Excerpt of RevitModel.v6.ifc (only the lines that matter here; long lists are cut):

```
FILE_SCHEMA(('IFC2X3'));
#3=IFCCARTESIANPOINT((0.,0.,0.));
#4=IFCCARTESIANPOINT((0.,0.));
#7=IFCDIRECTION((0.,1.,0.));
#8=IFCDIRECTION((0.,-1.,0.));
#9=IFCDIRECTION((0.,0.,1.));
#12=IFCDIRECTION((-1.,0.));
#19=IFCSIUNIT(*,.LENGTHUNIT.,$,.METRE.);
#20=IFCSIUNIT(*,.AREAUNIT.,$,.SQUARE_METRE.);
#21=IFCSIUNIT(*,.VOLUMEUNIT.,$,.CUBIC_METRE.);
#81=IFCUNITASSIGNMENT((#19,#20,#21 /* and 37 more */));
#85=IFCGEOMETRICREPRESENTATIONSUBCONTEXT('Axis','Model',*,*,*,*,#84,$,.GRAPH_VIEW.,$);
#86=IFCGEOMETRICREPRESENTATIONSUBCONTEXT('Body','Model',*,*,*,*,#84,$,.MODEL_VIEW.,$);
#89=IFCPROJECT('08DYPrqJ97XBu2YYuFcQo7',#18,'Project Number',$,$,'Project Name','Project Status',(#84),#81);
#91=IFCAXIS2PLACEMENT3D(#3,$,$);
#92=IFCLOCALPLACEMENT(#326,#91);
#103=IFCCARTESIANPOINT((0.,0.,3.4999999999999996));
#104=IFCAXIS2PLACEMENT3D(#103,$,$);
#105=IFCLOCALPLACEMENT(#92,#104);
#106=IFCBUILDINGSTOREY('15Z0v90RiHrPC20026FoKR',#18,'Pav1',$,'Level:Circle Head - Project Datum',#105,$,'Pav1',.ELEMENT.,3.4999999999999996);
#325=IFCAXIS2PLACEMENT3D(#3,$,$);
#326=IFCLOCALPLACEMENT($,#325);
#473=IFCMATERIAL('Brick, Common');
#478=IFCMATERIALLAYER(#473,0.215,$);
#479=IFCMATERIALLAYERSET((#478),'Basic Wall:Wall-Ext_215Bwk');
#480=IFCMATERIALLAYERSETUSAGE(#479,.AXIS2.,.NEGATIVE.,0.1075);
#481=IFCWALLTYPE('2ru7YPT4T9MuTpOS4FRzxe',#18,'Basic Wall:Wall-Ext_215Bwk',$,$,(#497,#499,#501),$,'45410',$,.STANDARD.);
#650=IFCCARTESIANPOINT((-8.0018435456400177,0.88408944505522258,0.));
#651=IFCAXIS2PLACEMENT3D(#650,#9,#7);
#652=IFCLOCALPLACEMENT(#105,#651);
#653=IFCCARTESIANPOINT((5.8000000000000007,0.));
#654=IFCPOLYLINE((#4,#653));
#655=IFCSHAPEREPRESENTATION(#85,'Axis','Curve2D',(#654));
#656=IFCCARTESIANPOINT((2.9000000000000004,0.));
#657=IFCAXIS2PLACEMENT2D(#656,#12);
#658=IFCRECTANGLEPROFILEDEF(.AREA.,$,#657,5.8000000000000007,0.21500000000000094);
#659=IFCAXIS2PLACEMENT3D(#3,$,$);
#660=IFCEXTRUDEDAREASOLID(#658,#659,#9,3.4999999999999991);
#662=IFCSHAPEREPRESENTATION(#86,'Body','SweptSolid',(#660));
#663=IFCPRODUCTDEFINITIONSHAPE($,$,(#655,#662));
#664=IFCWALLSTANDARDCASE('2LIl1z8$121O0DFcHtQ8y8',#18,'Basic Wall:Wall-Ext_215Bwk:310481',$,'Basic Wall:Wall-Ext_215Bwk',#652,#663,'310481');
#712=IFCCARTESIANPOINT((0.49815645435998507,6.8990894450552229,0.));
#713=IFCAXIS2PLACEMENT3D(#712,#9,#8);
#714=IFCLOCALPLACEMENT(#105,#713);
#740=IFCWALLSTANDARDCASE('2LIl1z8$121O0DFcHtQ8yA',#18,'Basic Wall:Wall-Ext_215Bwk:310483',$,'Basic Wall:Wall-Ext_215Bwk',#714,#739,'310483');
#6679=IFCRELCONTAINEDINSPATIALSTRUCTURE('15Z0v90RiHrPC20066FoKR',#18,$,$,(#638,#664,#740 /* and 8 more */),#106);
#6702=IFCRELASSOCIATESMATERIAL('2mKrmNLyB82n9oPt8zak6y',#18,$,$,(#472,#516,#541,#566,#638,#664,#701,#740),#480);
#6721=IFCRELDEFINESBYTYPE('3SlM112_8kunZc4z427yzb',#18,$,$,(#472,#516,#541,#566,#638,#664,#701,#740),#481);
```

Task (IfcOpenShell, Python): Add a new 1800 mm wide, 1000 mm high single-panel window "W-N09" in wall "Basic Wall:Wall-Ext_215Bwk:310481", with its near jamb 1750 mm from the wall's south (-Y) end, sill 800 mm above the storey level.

```python
import numpy as np
import ifcopenshell
import ifcopenshell.api.feature
import ifcopenshell.api.geometry
import ifcopenshell.api.root
import ifcopenshell.api.spatial
import ifcopenshell.api.type
import ifcopenshell.geom
import ifcopenshell.util.element
import ifcopenshell.util.placement
import ifcopenshell.util.representation
import ifcopenshell.util.shape
import ifcopenshell.util.unit

model = ifcopenshell.open("RevitModel.v6.ifc")
unit_scale = ifcopenshell.util.unit.calculate_unit_scale(model)
settings = ifcopenshell.geom.settings()


def volume(element):
    """Net volume in cubic metres, openings subtracted."""
    shape = ifcopenshell.geom.create_shape(settings, element)
    return ifcopenshell.util.shape.get_volume(shape.geometry)


wall = model.by_id(664)
storey = ifcopenshell.util.element.get_container(wall, ifc_class="IfcBuildingStorey")
context = ifcopenshell.util.representation.get_context(model, "Model", "Body", "MODEL_VIEW")
before = volume(wall)

width, height, from_end, sill = 1.8, 1, 1.75, 0.8  # metres

# The wall runs along its own X axis, and the end named is its -X end.
wall_shape = ifcopenshell.geom.create_shape(settings, wall)
x, y, z = ifcopenshell.util.shape.get_vertices(wall_shape.geometry).T
start = x.min() + from_end
face, thickness = float(y.min()), float(y.max() - y.min())
wall_matrix = ifcopenshell.util.placement.get_local_placement(wall.ObjectPlacement)
level = ifcopenshell.util.placement.get_local_placement(storey.ObjectPlacement)[2, 3]


def in_wall(x, y):
    """Placement at x, y metres in the wall's axes, at sill height."""
    matrix = wall_matrix.copy()
    matrix[:, 3] = wall_matrix @ np.array([x / unit_scale, y / unit_scale, 0.0, 1.0])
    matrix[2, 3] = level + sill / unit_scale
    return matrix


# Opening: a box that overshoots both wall faces by 50 mm.
opening = ifcopenshell.api.root.create_entity(model, ifc_class="IfcOpeningElement")
box = ifcopenshell.api.geometry.add_wall_representation(
    model, context=context, length=width, height=height, thickness=thickness + 0.1
)
ifcopenshell.api.geometry.assign_representation(model, product=opening, representation=box)
ifcopenshell.api.geometry.edit_object_placement(model, product=opening, matrix=in_wall(start, face - 0.05), is_si=False)
ifcopenshell.api.feature.add_feature(model, feature=opening, element=wall)

window = ifcopenshell.api.root.create_entity(model, ifc_class="IfcWindow", name="W-N09")
window.OverallWidth, window.OverallHeight = width / unit_scale, height / unit_scale
body = ifcopenshell.api.geometry.add_window_representation(
    model,
    context=context,
    overall_width=window.OverallWidth,
    overall_height=window.OverallHeight,
    partition_type="SINGLE_PANEL",
)
ifcopenshell.api.geometry.assign_representation(model, product=window, representation=body)
ifcopenshell.api.spatial.assign_container(model, products=[window], relating_structure=storey)
fills = ifcopenshell.api.feature.add_filling(model, opening=opening, element=window)
fills.OwnerHistory = window.OwnerHistory  # required in IFC2X3

# IFC2X3 keeps the operation on the window style.
style = ifcopenshell.api.root.create_entity(model, ifc_class="IfcWindowStyle", name="W-N09")
style.OperationType, style.ConstructionType = "SINGLE_PANEL", "NOTDEFINED"
style.ParameterTakesPrecedence = style.Sizeable = False
ifcopenshell.api.type.assign_type(model, related_objects=[window], relating_type=style)

# Centre the window in the wall's thickness.
ifcopenshell.api.geometry.edit_object_placement(model, product=window, matrix=in_wall(start, face), is_si=False)
window_shape = ifcopenshell.geom.create_shape(settings, window)
depth = ifcopenshell.util.shape.get_vertices(window_shape.geometry)[:, 1]
offset = face + thickness / 2 - (depth.min() + depth.max()) / 2
ifcopenshell.api.geometry.edit_object_placement(model, product=window, matrix=in_wall(start, offset), is_si=False)

after = volume(wall)

print(f"wall volume {before:.3f} -> {after:.3f} m3")

model.write("RevitModel.v6_updated.ifc")
```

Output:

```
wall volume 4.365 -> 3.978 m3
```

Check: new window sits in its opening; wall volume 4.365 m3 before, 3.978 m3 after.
